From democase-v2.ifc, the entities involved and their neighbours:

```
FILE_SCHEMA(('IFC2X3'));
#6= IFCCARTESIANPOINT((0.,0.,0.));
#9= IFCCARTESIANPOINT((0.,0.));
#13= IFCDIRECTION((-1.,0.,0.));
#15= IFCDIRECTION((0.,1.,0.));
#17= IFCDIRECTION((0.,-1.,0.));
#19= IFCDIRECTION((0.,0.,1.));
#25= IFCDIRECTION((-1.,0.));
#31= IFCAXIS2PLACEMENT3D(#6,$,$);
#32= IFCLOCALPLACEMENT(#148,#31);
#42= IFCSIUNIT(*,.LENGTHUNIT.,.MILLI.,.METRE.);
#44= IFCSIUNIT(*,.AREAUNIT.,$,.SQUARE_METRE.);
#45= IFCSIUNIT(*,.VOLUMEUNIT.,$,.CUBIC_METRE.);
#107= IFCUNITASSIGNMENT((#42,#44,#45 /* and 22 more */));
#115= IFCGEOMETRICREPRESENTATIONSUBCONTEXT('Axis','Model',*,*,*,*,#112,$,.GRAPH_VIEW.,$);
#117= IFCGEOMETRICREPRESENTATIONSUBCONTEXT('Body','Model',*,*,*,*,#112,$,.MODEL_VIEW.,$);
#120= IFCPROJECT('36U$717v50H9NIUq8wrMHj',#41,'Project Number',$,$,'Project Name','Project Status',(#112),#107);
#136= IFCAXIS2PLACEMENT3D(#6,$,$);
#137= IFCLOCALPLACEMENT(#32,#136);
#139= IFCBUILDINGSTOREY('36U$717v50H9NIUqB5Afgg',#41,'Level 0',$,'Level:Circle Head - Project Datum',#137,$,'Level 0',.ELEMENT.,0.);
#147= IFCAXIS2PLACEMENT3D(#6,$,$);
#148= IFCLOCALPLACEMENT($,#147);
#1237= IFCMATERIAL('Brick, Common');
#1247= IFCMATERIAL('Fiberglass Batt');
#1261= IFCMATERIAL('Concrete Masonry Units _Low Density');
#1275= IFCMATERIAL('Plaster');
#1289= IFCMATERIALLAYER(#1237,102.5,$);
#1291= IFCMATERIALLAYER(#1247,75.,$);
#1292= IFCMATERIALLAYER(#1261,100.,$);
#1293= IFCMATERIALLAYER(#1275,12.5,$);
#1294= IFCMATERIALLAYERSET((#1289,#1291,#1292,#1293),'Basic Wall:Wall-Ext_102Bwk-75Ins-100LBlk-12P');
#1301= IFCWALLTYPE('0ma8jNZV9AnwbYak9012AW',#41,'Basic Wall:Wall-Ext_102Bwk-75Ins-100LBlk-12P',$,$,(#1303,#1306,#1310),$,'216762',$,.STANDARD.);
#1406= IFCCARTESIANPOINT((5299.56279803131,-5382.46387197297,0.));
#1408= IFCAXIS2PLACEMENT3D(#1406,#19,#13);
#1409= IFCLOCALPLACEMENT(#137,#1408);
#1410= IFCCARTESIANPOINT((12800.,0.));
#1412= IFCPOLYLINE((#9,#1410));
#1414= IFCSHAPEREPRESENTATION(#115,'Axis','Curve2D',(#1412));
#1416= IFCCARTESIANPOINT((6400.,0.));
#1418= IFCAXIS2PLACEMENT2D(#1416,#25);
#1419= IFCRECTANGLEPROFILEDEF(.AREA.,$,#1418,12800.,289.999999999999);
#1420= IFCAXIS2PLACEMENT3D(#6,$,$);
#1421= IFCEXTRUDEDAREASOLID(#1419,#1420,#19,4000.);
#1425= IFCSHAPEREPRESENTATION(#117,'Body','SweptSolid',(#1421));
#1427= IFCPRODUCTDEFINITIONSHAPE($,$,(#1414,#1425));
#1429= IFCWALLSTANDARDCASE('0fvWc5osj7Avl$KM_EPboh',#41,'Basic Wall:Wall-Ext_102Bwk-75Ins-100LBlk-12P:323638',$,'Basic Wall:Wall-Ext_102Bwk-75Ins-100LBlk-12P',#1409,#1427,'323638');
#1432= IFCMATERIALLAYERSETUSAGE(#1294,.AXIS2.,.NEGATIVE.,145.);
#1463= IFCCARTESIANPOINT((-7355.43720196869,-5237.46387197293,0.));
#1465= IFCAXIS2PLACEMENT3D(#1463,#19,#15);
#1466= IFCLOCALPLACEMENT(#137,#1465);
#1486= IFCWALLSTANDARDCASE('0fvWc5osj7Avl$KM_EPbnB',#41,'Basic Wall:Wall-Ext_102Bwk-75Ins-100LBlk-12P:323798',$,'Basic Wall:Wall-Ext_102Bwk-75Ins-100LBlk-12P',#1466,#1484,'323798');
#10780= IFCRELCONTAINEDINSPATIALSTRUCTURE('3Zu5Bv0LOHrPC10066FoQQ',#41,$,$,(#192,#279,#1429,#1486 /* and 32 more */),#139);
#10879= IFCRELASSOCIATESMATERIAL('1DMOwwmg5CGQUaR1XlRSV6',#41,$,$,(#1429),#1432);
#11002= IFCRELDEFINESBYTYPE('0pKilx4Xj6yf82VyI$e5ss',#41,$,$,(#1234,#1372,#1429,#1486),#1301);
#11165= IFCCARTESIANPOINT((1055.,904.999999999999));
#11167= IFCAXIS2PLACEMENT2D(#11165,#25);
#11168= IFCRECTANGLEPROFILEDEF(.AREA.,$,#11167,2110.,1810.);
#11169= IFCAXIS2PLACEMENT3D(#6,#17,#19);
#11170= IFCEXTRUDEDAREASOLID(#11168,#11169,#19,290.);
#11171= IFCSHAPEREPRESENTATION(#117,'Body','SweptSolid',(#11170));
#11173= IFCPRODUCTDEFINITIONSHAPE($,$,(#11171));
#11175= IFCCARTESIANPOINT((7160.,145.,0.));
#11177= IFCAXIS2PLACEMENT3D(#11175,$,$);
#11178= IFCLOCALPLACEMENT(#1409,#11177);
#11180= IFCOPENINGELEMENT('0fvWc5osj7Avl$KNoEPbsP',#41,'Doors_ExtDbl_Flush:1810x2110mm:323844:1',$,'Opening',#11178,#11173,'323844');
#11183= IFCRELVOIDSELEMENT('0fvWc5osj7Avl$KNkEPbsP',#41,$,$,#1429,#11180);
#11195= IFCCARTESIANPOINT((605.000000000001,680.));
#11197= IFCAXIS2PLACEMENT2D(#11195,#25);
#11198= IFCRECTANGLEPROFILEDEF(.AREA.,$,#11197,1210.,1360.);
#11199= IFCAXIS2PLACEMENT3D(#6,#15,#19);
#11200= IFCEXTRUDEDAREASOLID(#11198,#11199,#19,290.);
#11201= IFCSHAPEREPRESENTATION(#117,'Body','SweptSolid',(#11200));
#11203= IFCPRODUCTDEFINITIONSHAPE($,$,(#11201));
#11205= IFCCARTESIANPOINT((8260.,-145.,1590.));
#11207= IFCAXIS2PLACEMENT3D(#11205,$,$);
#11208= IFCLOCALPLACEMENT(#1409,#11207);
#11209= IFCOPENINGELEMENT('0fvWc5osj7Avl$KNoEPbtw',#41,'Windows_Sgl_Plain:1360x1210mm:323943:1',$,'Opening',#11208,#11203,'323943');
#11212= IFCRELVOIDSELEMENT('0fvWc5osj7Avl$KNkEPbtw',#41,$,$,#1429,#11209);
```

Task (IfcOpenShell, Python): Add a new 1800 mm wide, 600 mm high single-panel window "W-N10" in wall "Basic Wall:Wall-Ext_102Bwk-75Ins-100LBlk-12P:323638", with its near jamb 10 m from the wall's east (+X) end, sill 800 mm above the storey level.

```python
import numpy as np
import ifcopenshell
import ifcopenshell.api.feature
import ifcopenshell.api.geometry
import ifcopenshell.api.root
import ifcopenshell.api.spatial
import ifcopenshell.api.type
import ifcopenshell.geom
import ifcopenshell.util.element
import ifcopenshell.util.placement
import ifcopenshell.util.representation
import ifcopenshell.util.shape
import ifcopenshell.util.unit

model = ifcopenshell.open("democase-v2.ifc")
unit_scale = ifcopenshell.util.unit.calculate_unit_scale(model)
settings = ifcopenshell.geom.settings()


def volume(element):
    """Net volume in cubic metres, openings subtracted."""
    shape = ifcopenshell.geom.create_shape(settings, element)
    return ifcopenshell.util.shape.get_volume(shape.geometry)


wall = model.by_guid("0fvWc5osj7Avl$KM_EPboh")
storey = ifcopenshell.util.element.get_container(wall, ifc_class="IfcBuildingStorey")
context = ifcopenshell.util.representation.get_context(model, "Model", "Body", "MODEL_VIEW")
before = volume(wall)

width, height, from_end, sill = 1.8, 0.6, 10, 0.8  # metres

# The wall runs along its own X axis, and the end named is its -X end.
wall_shape = ifcopenshell.geom.create_shape(settings, wall)
x, y, z = ifcopenshell.util.shape.get_vertices(wall_shape.geometry).T
start = x.min() + from_end
face, thickness = float(y.min()), float(y.max() - y.min())
wall_matrix = ifcopenshell.util.placement.get_local_placement(wall.ObjectPlacement)
level = ifcopenshell.util.placement.get_local_placement(storey.ObjectPlacement)[2, 3]


def in_wall(x, y):
    """Placement at x, y metres in the wall's axes, at sill height."""
    matrix = wall_matrix.copy()
    matrix[:, 3] = wall_matrix @ np.array([x / unit_scale, y / unit_scale, 0.0, 1.0])
    matrix[2, 3] = level + sill / unit_scale
    return matrix


# Opening: a box that overshoots both wall faces by 50 mm.
opening = ifcopenshell.api.root.create_entity(model, ifc_class="IfcOpeningElement")
box = ifcopenshell.api.geometry.add_wall_representation(
    model, context=context, length=width, height=height, thickness=thickness + 0.1
)
ifcopenshell.api.geometry.assign_representation(model, product=opening, representation=box)
ifcopenshell.api.geometry.edit_object_placement(model, product=opening, matrix=in_wall(start, face - 0.05), is_si=False)
ifcopenshell.api.feature.add_feature(model, feature=opening, element=wall)

window = ifcopenshell.api.root.create_entity(model, ifc_class="IfcWindow", name="W-N10")
window.OverallWidth, window.OverallHeight = width / unit_scale, height / unit_scale
body = ifcopenshell.api.geometry.add_window_representation(
    model,
    context=context,
    overall_width=window.OverallWidth,
    overall_height=window.OverallHeight,
    partition_type="SINGLE_PANEL",
)
ifcopenshell.api.geometry.assign_representation(model, product=window, representation=body)
ifcopenshell.api.spatial.assign_container(model, products=[window], relating_structure=storey)
fills = ifcopenshell.api.feature.add_filling(model, opening=opening, element=window)
fills.OwnerHistory = window.OwnerHistory  # required in IFC2X3

# IFC2X3 keeps the operation on the window style.
style = ifcopenshell.api.root.create_entity(model, ifc_class="IfcWindowStyle", name="W-N10")
style.OperationType, style.ConstructionType = "SINGLE_PANEL", "NOTDEFINED"
style.ParameterTakesPrecedence = style.Sizeable = False
ifcopenshell.api.type.assign_type(model, related_objects=[window], relating_type=style)

# Centre the window in the wall's thickness.
ifcopenshell.api.geometry.edit_object_placement(model, product=window, matrix=in_wall(start, face), is_si=False)
window_shape = ifcopenshell.geom.create_shape(settings, window)
depth = ifcopenshell.util.shape.get_vertices(window_shape.geometry)[:, 1]
offset = face + thickness / 2 - (depth.min() + depth.max()) / 2
ifcopenshell.api.geometry.edit_object_placement(model, product=window, matrix=in_wall(start, offset), is_si=False)

after = volume(wall)

print(f"wall volume {before:.3f} -> {after:.3f} m3")

model.write("democase-v2-out.ifc")
```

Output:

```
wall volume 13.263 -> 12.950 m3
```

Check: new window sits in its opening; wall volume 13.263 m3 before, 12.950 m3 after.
